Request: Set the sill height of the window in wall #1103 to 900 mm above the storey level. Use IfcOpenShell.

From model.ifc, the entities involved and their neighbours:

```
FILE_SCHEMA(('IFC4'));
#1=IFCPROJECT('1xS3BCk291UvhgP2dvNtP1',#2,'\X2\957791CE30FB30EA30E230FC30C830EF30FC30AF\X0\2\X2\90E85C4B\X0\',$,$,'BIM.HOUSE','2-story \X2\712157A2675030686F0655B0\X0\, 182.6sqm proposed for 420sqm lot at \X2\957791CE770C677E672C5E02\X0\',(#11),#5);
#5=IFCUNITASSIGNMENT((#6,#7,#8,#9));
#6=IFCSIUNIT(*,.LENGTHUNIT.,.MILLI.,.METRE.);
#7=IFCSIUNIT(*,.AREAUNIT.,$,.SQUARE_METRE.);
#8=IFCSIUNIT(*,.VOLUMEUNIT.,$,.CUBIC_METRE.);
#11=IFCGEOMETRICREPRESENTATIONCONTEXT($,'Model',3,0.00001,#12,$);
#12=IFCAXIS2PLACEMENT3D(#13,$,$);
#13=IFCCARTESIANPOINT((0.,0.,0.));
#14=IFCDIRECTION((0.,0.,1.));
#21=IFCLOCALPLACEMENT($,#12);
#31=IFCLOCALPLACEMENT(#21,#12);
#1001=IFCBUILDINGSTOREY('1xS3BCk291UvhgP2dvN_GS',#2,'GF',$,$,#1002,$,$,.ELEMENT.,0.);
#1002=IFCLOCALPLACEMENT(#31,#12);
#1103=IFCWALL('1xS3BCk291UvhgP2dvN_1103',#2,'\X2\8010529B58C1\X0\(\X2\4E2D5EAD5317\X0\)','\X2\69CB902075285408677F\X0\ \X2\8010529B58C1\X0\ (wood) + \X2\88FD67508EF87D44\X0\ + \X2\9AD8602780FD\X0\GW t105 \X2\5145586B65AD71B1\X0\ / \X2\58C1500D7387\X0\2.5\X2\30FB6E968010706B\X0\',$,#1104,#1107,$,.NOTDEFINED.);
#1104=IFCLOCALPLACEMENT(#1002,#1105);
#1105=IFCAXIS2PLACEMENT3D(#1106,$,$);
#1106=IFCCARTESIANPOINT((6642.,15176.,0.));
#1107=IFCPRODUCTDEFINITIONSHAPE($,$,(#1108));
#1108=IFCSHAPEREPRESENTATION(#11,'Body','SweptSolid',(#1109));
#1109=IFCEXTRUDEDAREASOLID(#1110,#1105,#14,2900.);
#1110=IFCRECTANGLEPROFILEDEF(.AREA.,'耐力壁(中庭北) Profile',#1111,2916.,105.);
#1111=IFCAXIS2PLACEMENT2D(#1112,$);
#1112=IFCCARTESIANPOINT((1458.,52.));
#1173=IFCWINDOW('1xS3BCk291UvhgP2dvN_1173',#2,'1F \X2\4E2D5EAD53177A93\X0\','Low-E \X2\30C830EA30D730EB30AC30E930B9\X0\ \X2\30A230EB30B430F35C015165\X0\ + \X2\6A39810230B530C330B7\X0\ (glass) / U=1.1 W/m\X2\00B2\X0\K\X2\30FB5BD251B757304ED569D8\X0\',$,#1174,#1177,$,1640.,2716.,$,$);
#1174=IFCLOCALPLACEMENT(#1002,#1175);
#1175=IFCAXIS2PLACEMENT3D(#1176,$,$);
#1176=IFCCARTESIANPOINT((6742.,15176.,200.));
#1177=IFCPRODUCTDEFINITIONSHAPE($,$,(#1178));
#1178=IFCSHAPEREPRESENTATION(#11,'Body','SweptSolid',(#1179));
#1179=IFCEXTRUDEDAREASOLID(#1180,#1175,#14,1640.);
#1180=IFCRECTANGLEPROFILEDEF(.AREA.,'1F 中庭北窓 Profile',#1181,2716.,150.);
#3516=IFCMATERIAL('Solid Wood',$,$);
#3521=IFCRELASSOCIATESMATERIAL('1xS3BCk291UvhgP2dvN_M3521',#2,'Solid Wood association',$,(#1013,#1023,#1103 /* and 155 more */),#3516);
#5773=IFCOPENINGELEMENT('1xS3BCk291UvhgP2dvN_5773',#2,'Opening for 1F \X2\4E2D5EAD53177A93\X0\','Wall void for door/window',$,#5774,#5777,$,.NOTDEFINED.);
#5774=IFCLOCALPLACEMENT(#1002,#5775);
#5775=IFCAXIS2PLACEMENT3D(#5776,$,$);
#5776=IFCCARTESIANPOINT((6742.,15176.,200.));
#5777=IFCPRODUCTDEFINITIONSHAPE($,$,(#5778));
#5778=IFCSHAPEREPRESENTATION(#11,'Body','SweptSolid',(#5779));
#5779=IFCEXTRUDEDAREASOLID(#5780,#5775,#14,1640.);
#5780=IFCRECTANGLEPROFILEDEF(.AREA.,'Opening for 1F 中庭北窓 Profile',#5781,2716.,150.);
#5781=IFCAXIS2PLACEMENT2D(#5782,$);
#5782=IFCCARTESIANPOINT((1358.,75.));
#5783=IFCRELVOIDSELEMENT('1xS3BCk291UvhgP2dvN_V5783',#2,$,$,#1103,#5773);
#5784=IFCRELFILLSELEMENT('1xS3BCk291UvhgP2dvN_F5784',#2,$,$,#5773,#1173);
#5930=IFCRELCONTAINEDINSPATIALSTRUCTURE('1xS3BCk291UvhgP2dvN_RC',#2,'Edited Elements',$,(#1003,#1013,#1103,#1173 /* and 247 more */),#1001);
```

```python
import numpy as np
import ifcopenshell
import ifcopenshell.api.geometry
import ifcopenshell.geom
import ifcopenshell.util.element
import ifcopenshell.util.placement
import ifcopenshell.util.shape
import ifcopenshell.util.unit

model = ifcopenshell.open("model.ifc")
unit_scale = ifcopenshell.util.unit.calculate_unit_scale(model)

window = model.by_id(1173)
opening = window.FillsVoids[0].RelatingOpeningElement
storey = ifcopenshell.util.element.get_container(window, ifc_class="IfcBuildingStorey")
level = ifcopenshell.util.placement.get_local_placement(storey.ObjectPlacement)[2, 3]

# The opening's origin need not be at the sill, so measure its lowest point.
shape = ifcopenshell.geom.create_shape(ifcopenshell.geom.settings(), opening)
bottom = ifcopenshell.util.shape.get_shape_bottom_elevation(shape, shape.geometry) / unit_scale
dz = level + 900.0 - bottom

shift = np.array([0.0, 0.0, dz])
# The window is not placed relative to its opening, so move both.
for product in (opening, window):
    matrix = ifcopenshell.util.placement.get_local_placement(product.ObjectPlacement)
    matrix[:3, 3] += shift
    ifcopenshell.api.geometry.edit_object_placement(model, product=product, matrix=matrix, is_si=False)

print(f"moved by {dz * unit_scale:+.3f} m")

model.write("model_updated.ifc")
```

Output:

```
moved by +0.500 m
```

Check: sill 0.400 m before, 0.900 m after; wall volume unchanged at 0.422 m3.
